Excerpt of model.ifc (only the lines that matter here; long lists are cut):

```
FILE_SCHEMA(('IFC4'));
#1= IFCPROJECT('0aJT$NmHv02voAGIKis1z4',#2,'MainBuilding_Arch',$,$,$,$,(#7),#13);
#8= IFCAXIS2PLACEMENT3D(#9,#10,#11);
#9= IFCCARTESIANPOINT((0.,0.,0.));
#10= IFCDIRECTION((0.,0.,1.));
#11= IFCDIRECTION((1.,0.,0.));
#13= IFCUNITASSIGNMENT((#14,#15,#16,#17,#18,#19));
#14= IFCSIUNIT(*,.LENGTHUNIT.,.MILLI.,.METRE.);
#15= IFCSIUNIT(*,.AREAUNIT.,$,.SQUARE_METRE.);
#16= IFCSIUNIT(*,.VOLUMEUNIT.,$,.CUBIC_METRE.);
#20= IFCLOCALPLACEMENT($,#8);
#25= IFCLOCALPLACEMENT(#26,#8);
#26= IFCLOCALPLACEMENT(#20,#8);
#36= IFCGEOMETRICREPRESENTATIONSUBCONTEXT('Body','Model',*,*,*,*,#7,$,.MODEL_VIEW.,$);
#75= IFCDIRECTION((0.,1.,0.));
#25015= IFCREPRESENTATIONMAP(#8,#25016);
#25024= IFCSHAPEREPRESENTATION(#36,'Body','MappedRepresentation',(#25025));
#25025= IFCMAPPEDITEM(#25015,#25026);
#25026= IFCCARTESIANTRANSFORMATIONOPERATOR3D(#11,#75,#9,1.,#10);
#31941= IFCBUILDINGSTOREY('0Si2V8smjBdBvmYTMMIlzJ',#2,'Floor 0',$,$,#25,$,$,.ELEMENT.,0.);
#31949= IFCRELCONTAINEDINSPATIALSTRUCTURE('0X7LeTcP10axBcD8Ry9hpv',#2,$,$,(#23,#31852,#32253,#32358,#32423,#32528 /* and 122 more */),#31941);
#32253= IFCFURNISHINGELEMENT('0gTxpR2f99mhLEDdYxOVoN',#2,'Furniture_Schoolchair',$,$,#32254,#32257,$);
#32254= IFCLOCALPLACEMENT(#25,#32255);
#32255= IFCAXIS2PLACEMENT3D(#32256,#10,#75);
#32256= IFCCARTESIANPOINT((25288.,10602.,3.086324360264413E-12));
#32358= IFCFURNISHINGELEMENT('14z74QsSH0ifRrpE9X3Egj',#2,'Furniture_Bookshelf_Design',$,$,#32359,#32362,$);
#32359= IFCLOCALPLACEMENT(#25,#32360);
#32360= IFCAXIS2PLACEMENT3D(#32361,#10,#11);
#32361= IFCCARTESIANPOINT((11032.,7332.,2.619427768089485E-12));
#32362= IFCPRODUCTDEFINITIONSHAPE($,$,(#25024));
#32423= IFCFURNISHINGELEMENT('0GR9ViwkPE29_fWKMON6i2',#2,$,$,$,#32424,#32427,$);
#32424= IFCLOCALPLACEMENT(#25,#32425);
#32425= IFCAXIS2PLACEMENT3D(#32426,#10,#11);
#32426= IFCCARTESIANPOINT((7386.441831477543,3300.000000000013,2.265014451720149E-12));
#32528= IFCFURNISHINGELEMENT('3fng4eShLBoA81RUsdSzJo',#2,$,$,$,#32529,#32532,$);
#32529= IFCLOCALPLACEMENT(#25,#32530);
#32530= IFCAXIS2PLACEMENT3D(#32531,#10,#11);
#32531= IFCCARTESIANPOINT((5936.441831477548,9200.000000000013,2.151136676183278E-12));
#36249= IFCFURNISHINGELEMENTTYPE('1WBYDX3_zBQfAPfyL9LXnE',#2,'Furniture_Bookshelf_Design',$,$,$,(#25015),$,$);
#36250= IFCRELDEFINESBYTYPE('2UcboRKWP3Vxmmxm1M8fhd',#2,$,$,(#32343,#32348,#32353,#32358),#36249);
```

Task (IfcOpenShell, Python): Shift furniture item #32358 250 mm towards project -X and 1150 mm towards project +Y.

```python
import ifcopenshell
import ifcopenshell.api.geometry
import ifcopenshell.util.placement
import ifcopenshell.util.unit

model = ifcopenshell.open("model.ifc")
unit_scale = ifcopenshell.util.unit.calculate_unit_scale(model)

item = model.by_guid("14z74QsSH0ifRrpE9X3Egj")
matrix = ifcopenshell.util.placement.get_local_placement(item.ObjectPlacement)
matrix[0, 3] -= 0.25 / unit_scale
matrix[1, 3] += 1.15 / unit_scale
ifcopenshell.api.geometry.edit_object_placement(model, product=item, matrix=matrix, is_si=False)

print(ifcopenshell.util.placement.get_local_placement(item.ObjectPlacement).round(3) + 0.0)

model.write("model_v2.ifc")
```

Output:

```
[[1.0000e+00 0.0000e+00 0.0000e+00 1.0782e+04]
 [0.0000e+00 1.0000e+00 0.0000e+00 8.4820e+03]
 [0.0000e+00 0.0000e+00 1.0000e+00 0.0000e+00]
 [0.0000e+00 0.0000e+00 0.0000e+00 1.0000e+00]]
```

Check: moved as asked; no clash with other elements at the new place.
